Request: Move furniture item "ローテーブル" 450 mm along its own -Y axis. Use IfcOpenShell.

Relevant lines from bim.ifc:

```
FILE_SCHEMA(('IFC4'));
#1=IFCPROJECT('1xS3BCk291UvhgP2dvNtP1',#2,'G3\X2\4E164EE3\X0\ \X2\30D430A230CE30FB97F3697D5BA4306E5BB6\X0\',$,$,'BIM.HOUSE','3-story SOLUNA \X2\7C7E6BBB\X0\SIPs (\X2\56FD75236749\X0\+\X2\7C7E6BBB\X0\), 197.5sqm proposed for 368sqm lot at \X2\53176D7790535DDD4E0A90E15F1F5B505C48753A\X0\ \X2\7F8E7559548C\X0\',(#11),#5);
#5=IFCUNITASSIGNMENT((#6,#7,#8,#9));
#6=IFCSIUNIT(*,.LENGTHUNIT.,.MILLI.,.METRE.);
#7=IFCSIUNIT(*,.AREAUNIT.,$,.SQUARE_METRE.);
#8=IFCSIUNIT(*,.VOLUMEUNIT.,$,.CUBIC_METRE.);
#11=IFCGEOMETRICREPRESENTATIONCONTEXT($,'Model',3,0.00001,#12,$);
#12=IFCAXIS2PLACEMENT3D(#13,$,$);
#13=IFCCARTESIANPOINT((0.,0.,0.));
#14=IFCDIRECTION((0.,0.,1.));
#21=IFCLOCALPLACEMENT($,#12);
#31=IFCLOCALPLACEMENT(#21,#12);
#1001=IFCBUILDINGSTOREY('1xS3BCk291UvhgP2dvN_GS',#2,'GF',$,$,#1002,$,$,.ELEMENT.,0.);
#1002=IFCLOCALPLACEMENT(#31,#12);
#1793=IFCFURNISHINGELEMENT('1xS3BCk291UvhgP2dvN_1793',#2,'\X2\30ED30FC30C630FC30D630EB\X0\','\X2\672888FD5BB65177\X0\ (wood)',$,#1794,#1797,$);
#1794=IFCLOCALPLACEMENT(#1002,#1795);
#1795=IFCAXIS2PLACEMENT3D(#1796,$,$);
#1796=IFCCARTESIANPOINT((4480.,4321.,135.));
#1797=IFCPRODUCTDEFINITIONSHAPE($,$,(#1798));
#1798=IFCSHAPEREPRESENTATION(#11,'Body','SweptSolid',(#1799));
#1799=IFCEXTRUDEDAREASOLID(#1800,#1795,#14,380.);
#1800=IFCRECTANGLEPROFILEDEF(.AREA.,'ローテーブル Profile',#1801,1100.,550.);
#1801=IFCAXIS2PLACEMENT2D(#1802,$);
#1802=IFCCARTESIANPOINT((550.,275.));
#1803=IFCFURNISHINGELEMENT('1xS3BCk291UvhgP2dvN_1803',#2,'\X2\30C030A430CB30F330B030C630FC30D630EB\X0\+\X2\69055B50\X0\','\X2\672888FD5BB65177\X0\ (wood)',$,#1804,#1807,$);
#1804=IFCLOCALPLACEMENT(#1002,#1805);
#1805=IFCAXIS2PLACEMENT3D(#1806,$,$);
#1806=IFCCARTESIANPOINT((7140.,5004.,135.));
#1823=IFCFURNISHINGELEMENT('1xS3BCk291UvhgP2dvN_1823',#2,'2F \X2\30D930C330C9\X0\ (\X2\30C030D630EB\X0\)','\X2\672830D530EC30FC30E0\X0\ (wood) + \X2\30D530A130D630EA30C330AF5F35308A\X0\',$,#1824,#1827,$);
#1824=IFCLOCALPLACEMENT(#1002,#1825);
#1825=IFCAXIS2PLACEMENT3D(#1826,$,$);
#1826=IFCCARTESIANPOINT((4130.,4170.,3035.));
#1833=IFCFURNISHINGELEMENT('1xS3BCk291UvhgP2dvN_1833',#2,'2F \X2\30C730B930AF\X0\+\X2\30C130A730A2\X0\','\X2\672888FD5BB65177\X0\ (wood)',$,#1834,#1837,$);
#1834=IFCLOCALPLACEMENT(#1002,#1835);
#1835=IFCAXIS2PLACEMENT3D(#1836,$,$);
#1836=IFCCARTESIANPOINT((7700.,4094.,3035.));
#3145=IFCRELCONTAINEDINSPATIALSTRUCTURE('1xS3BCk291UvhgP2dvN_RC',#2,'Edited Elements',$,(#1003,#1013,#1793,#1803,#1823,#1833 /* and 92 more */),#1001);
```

```python
import ifcopenshell
import ifcopenshell.api.geometry
import ifcopenshell.util.placement
import ifcopenshell.util.unit

model = ifcopenshell.open("bim.ifc")
unit_scale = ifcopenshell.util.unit.calculate_unit_scale(model)

item = model.by_guid("1xS3BCk291UvhgP2dvN_1793")
matrix = ifcopenshell.util.placement.get_local_placement(item.ObjectPlacement)
matrix[:3, 3] -= matrix[:3, 1] * 0.45 / unit_scale
ifcopenshell.api.geometry.edit_object_placement(model, product=item, matrix=matrix, is_si=False)

print(ifcopenshell.util.placement.get_local_placement(item.ObjectPlacement).round(3) + 0.0)

model.write("bim-out.ifc")
```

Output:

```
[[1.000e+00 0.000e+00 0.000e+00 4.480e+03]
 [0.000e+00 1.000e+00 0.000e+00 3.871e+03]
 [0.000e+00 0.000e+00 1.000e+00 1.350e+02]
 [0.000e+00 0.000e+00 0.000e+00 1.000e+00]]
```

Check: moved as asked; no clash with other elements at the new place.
